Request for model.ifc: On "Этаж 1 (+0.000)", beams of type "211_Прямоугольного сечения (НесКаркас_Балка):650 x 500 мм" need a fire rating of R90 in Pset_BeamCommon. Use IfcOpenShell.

First a look at what the model holds.

```python
import ifcopenshell
import ifcopenshell.util.element

model = ifcopenshell.open("model.ifc")
print(model.schema)
storey = next(s for s in model.by_type("IfcBuildingStorey") if s.Name == "Этаж 1 (+0.000)")
beams = [e for e in ifcopenshell.util.element.get_decomposition(storey) if e.is_a("IfcBeam")]
seen = {}
for e in beams:
    element_type = ifcopenshell.util.element.get_type(e)
    key = (element_type.Name if element_type != e and element_type else None, ifcopenshell.util.element.get_pset(e, "Pset_BeamCommon", "FireRating"))
    seen[key] = seen.get(key, 0) + 1
for (name, value), count in sorted(seen.items(), key=str):
    print(count, "x", name, "|", value)
```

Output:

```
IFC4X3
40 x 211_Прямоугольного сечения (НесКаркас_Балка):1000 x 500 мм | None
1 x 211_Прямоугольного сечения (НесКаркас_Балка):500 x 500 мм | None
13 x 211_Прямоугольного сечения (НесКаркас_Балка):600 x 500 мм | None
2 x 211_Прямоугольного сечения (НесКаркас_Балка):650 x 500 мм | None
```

```python
import ifcopenshell
import ifcopenshell.api.pset
import ifcopenshell.util.element

model = ifcopenshell.open("model.ifc")

storey = next(s for s in model.by_type("IfcBuildingStorey") if s.Name == "Этаж 1 (+0.000)")
beams = [e for e in ifcopenshell.util.element.get_decomposition(storey) if e.is_a("IfcBeam")]

count = 0
for e in beams:
    element_type = ifcopenshell.util.element.get_type(e)
    if element_type in (None, e) or element_type.Name != "211_Прямоугольного сечения (НесКаркас_Балка):650 x 500 мм":
        continue
    # add_pset returns the element's existing set when there is one.
    pset = ifcopenshell.api.pset.add_pset(model, product=e, name="Pset_BeamCommon")
    ifcopenshell.api.pset.edit_pset(model, pset=pset, properties={"FireRating": "R90"})
    count += 1

print(count, "beams updated")

model.write("model_updated.ifc")
```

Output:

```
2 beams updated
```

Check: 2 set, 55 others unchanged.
